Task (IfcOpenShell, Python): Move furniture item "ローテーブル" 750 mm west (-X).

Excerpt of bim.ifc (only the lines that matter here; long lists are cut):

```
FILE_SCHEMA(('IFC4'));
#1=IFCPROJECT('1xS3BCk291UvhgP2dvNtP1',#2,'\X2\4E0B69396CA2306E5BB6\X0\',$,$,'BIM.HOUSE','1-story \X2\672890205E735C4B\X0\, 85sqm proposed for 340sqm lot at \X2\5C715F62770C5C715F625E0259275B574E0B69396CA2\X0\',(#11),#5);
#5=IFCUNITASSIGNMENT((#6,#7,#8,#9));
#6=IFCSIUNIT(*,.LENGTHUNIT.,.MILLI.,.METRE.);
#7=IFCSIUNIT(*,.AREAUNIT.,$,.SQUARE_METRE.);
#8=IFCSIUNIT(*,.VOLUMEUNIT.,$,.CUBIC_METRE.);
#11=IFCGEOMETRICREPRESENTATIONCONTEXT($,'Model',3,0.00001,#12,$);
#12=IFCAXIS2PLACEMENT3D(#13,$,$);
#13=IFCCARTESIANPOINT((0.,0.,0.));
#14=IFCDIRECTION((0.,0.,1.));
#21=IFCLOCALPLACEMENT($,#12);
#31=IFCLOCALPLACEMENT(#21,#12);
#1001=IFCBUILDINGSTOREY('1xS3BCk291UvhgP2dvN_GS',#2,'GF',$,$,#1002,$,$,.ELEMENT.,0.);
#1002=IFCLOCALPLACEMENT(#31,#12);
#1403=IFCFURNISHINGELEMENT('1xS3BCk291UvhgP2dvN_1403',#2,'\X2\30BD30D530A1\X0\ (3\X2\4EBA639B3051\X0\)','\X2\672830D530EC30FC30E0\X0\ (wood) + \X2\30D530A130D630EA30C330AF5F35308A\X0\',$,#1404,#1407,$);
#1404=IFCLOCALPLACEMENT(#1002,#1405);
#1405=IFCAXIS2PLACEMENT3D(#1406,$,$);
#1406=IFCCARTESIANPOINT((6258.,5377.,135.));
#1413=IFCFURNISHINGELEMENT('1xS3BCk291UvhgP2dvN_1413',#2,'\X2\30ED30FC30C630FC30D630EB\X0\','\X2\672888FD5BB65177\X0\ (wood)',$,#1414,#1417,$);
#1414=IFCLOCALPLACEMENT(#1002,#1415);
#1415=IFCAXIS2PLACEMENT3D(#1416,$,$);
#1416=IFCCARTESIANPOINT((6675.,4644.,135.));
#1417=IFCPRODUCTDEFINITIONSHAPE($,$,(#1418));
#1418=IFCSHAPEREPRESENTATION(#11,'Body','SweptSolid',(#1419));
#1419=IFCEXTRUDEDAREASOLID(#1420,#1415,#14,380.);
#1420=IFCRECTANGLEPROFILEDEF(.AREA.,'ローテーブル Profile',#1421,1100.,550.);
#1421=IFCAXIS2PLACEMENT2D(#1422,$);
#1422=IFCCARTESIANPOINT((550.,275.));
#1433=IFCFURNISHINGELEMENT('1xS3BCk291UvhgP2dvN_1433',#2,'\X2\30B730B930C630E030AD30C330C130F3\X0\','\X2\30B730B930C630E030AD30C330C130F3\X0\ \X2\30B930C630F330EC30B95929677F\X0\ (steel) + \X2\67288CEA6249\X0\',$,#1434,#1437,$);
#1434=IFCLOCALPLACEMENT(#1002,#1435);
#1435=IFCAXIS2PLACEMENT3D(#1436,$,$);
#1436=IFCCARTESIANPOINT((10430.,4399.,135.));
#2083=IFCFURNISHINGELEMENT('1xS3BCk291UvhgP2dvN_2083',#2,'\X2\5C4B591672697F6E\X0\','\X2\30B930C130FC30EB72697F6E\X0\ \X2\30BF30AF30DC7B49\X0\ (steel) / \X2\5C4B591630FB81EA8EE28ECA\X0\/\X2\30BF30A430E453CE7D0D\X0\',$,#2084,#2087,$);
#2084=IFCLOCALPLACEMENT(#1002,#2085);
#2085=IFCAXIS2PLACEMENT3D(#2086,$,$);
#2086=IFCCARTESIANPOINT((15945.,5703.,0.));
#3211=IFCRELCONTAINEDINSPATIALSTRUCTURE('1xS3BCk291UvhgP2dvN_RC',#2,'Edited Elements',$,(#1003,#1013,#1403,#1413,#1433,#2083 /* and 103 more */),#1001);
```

```python
import ifcopenshell
import ifcopenshell.api.geometry
import ifcopenshell.util.placement

model = ifcopenshell.open("bim.ifc")

item = model.by_guid("1xS3BCk291UvhgP2dvN_1413")
matrix = ifcopenshell.util.placement.get_local_placement(item.ObjectPlacement)
matrix[0, 3] -= 750.0
ifcopenshell.api.geometry.edit_object_placement(model, product=item, matrix=matrix, is_si=False)

print(ifcopenshell.util.placement.get_local_placement(item.ObjectPlacement).round(3) + 0.0)

model.write("bim_rev.ifc")
```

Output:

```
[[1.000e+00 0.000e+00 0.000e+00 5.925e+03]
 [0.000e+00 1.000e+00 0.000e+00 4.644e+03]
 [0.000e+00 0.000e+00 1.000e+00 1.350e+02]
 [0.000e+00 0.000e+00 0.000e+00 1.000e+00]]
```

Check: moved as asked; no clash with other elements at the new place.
